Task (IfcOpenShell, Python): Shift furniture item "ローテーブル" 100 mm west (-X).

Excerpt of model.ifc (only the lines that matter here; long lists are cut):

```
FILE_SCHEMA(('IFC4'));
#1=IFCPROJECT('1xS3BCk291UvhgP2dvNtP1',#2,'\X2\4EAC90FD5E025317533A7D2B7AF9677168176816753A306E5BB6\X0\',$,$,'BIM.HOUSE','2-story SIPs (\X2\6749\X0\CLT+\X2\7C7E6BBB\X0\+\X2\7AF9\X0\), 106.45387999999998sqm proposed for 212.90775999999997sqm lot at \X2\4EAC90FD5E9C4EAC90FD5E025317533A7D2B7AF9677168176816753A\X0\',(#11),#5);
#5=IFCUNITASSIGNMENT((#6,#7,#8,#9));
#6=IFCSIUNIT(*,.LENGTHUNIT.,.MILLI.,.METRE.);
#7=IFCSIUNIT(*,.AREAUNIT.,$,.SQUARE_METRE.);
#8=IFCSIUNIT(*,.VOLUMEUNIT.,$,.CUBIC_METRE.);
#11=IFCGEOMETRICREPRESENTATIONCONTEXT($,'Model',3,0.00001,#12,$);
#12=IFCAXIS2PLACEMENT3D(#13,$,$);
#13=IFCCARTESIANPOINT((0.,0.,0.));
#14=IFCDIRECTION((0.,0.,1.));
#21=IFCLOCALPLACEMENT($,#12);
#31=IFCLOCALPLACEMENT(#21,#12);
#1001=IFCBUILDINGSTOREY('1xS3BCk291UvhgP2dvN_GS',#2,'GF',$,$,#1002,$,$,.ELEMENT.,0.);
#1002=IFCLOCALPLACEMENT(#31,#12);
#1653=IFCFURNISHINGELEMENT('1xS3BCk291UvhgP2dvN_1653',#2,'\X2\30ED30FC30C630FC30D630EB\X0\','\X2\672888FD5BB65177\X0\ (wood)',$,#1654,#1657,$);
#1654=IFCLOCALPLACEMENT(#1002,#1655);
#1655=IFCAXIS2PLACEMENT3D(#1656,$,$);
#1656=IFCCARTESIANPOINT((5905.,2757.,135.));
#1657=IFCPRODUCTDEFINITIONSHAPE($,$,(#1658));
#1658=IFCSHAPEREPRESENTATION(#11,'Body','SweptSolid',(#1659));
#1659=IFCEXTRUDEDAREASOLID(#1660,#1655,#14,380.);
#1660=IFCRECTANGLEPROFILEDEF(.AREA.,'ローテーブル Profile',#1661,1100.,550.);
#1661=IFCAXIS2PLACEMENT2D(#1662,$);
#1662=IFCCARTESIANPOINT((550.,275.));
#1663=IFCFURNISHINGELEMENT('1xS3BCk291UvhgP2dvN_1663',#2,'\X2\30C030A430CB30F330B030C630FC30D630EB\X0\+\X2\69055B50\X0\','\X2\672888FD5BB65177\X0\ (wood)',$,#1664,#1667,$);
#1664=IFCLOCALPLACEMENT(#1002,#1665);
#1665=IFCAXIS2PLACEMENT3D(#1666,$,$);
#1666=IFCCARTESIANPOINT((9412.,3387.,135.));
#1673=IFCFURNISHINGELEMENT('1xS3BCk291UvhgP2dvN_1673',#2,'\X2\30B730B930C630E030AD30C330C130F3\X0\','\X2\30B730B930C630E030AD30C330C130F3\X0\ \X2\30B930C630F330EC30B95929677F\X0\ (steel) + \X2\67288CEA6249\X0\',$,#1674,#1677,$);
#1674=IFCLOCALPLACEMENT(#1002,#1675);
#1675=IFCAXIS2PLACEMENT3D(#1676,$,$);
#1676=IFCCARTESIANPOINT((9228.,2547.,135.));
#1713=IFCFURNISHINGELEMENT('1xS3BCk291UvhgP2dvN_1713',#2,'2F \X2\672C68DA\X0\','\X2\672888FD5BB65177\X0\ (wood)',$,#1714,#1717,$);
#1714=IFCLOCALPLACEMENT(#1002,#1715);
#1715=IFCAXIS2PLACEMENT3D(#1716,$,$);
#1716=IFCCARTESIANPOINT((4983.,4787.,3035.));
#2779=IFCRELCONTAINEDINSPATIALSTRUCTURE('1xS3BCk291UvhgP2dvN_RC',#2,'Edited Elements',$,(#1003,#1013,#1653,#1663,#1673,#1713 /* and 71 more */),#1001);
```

```python
import ifcopenshell
import ifcopenshell.api.geometry
import ifcopenshell.util.placement

model = ifcopenshell.open("model.ifc")

item = model.by_guid("1xS3BCk291UvhgP2dvN_1653")
matrix = ifcopenshell.util.placement.get_local_placement(item.ObjectPlacement)
matrix[0, 3] -= 100.0
ifcopenshell.api.geometry.edit_object_placement(model, product=item, matrix=matrix, is_si=False)

print(ifcopenshell.util.placement.get_local_placement(item.ObjectPlacement).round(3) + 0.0)

model.write("model-out.ifc")
```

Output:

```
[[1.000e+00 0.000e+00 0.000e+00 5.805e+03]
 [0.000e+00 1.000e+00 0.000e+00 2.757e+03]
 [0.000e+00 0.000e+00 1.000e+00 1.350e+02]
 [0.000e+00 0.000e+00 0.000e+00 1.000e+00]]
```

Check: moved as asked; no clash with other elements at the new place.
